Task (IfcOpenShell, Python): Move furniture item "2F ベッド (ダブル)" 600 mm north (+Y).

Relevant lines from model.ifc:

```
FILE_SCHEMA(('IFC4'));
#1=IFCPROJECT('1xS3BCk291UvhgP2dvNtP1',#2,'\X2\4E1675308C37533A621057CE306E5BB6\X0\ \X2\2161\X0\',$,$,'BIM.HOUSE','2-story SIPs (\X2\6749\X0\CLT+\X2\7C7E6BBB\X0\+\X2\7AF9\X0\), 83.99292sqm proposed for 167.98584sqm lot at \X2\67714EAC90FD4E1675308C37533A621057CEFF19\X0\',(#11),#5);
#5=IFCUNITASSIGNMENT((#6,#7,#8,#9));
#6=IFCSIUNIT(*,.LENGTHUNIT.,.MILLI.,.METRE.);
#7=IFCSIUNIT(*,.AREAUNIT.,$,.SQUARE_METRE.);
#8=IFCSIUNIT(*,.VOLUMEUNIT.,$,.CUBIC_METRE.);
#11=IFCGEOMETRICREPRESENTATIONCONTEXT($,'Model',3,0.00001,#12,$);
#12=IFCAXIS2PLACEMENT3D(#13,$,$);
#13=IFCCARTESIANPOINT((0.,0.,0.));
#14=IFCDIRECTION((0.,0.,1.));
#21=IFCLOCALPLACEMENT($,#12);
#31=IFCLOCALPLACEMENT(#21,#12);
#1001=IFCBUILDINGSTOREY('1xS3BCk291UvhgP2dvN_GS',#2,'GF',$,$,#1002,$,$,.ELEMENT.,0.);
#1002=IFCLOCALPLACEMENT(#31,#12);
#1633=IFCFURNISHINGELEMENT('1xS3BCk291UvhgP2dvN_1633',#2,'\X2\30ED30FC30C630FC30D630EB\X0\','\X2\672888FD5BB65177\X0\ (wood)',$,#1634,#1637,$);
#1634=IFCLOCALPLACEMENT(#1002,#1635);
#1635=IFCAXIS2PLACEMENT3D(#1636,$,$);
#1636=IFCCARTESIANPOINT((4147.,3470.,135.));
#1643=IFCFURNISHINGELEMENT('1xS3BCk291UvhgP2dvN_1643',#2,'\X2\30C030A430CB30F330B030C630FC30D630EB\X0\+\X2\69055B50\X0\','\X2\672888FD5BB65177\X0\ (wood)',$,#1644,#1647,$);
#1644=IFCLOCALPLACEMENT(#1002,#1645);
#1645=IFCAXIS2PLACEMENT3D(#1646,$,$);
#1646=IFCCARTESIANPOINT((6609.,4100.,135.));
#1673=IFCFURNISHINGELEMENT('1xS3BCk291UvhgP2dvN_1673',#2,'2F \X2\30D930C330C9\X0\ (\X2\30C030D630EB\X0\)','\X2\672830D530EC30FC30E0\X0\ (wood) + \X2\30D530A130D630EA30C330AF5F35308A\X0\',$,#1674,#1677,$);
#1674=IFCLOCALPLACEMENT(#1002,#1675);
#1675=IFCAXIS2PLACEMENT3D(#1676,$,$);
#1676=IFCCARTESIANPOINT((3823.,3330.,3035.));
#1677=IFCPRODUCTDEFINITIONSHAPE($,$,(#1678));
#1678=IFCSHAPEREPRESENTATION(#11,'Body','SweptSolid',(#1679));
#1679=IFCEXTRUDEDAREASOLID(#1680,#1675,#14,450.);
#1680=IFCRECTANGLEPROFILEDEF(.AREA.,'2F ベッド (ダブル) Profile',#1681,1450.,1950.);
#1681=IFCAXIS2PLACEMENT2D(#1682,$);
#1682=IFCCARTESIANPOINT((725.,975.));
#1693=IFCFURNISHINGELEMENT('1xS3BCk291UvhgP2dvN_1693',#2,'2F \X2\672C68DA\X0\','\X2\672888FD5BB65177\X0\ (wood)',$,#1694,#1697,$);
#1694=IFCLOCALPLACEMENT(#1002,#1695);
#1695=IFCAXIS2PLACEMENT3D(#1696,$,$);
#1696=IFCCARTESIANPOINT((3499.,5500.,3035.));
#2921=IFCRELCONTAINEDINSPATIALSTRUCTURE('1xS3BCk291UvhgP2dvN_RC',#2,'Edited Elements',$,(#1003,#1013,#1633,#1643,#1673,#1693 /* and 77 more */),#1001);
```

```python
import ifcopenshell
import ifcopenshell.api.geometry
import ifcopenshell.util.placement
import ifcopenshell.util.unit

model = ifcopenshell.open("model.ifc")
unit_scale = ifcopenshell.util.unit.calculate_unit_scale(model)

item = model.by_guid("1xS3BCk291UvhgP2dvN_1673")
matrix = ifcopenshell.util.placement.get_local_placement(item.ObjectPlacement)
matrix[1, 3] += 0.6 / unit_scale
ifcopenshell.api.geometry.edit_object_placement(model, product=item, matrix=matrix, is_si=False)

print(ifcopenshell.util.placement.get_local_placement(item.ObjectPlacement).round(3) + 0.0)

model.write("model-out.ifc")
```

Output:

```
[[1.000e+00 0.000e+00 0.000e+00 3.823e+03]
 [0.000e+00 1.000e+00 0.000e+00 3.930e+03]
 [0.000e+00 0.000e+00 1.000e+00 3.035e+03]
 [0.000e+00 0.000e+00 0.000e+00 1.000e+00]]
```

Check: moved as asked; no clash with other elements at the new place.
